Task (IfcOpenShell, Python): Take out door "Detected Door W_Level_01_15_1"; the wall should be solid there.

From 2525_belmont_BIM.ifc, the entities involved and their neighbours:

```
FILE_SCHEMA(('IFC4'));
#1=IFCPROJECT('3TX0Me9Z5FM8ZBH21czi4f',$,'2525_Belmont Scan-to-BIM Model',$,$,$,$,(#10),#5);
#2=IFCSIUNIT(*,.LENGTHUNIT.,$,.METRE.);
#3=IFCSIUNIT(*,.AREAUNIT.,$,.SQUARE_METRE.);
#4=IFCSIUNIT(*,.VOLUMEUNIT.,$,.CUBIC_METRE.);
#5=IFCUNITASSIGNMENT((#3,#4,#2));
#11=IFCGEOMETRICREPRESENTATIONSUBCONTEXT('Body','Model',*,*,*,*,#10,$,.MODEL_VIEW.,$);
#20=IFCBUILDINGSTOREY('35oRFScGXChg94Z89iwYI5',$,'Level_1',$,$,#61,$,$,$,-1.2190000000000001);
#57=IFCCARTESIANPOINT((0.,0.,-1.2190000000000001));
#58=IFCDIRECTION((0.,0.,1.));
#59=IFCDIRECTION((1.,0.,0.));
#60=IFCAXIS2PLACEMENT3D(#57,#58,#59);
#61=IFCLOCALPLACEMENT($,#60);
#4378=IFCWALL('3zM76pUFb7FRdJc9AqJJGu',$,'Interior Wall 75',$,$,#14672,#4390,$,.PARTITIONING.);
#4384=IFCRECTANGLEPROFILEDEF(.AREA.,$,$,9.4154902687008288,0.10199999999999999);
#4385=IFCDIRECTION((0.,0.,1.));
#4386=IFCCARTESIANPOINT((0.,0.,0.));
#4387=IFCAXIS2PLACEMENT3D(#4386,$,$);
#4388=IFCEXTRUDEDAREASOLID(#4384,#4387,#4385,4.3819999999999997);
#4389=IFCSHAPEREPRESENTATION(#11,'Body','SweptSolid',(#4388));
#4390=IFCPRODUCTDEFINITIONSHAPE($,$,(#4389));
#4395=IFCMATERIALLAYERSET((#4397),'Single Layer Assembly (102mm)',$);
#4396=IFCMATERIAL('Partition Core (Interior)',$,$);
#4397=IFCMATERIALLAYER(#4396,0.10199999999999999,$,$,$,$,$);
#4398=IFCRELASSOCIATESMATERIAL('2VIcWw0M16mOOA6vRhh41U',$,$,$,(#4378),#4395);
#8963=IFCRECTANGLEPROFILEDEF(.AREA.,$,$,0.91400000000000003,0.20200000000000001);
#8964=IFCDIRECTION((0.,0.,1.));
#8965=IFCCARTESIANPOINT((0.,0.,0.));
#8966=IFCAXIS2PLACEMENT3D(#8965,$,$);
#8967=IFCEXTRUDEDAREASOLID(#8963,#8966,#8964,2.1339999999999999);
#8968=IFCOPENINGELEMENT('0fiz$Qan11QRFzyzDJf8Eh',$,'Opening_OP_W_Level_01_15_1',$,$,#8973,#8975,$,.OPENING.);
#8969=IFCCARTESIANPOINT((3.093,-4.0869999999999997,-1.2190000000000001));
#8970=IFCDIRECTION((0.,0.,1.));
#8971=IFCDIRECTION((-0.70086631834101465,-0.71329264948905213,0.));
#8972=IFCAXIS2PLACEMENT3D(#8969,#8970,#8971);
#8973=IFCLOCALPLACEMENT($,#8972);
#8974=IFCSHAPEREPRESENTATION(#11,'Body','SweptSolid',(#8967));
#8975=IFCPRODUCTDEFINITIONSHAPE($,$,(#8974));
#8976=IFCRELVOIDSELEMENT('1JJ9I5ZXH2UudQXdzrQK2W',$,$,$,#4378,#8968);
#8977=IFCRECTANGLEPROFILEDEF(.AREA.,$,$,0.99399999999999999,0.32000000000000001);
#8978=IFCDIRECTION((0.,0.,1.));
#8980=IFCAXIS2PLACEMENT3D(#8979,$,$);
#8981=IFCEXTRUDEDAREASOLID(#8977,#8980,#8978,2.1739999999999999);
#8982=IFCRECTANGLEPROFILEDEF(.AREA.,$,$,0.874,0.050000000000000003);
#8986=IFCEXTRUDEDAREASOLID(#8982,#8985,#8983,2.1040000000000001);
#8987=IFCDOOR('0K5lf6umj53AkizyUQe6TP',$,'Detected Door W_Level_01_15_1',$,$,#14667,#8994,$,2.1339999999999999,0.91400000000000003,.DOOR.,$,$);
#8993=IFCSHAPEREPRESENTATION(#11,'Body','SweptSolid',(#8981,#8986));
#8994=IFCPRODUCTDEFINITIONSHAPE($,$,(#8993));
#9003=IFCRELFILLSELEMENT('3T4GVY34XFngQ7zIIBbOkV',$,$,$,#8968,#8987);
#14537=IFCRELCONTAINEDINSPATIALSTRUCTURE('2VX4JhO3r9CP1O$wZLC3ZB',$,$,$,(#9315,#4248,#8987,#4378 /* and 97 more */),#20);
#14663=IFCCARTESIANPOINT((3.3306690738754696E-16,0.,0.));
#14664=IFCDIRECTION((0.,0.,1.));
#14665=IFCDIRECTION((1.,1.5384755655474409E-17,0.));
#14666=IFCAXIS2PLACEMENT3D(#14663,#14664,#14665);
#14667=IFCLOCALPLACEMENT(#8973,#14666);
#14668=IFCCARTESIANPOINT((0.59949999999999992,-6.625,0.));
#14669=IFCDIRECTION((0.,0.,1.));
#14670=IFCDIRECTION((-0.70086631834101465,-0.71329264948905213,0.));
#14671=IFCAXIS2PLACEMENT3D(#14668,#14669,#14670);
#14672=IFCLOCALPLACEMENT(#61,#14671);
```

```python
import ifcopenshell
import ifcopenshell.api.feature
import ifcopenshell.api.root
import ifcopenshell.geom
import ifcopenshell.util.shape

model = ifcopenshell.open("2525_belmont_BIM.ifc")
settings = ifcopenshell.geom.settings()


def volume(element):
    """Net volume in cubic metres, openings subtracted."""
    shape = ifcopenshell.geom.create_shape(settings, element)
    return ifcopenshell.util.shape.get_volume(shape.geometry)


door = model.by_guid("0K5lf6umj53AkizyUQe6TP")
opening = door.FillsVoids[0].RelatingOpeningElement
wall = opening.VoidsElements[0].RelatingBuildingElement
before = volume(wall)

ifcopenshell.api.root.remove_product(model, product=door)
ifcopenshell.api.feature.remove_feature(model, feature=opening)

after = volume(wall)

print(f"wall volume {before:.3f} -> {after:.3f} m3")

model.write("2525_belmont_BIM_v2.ifc")
```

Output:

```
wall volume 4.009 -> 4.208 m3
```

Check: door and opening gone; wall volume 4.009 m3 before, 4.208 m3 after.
